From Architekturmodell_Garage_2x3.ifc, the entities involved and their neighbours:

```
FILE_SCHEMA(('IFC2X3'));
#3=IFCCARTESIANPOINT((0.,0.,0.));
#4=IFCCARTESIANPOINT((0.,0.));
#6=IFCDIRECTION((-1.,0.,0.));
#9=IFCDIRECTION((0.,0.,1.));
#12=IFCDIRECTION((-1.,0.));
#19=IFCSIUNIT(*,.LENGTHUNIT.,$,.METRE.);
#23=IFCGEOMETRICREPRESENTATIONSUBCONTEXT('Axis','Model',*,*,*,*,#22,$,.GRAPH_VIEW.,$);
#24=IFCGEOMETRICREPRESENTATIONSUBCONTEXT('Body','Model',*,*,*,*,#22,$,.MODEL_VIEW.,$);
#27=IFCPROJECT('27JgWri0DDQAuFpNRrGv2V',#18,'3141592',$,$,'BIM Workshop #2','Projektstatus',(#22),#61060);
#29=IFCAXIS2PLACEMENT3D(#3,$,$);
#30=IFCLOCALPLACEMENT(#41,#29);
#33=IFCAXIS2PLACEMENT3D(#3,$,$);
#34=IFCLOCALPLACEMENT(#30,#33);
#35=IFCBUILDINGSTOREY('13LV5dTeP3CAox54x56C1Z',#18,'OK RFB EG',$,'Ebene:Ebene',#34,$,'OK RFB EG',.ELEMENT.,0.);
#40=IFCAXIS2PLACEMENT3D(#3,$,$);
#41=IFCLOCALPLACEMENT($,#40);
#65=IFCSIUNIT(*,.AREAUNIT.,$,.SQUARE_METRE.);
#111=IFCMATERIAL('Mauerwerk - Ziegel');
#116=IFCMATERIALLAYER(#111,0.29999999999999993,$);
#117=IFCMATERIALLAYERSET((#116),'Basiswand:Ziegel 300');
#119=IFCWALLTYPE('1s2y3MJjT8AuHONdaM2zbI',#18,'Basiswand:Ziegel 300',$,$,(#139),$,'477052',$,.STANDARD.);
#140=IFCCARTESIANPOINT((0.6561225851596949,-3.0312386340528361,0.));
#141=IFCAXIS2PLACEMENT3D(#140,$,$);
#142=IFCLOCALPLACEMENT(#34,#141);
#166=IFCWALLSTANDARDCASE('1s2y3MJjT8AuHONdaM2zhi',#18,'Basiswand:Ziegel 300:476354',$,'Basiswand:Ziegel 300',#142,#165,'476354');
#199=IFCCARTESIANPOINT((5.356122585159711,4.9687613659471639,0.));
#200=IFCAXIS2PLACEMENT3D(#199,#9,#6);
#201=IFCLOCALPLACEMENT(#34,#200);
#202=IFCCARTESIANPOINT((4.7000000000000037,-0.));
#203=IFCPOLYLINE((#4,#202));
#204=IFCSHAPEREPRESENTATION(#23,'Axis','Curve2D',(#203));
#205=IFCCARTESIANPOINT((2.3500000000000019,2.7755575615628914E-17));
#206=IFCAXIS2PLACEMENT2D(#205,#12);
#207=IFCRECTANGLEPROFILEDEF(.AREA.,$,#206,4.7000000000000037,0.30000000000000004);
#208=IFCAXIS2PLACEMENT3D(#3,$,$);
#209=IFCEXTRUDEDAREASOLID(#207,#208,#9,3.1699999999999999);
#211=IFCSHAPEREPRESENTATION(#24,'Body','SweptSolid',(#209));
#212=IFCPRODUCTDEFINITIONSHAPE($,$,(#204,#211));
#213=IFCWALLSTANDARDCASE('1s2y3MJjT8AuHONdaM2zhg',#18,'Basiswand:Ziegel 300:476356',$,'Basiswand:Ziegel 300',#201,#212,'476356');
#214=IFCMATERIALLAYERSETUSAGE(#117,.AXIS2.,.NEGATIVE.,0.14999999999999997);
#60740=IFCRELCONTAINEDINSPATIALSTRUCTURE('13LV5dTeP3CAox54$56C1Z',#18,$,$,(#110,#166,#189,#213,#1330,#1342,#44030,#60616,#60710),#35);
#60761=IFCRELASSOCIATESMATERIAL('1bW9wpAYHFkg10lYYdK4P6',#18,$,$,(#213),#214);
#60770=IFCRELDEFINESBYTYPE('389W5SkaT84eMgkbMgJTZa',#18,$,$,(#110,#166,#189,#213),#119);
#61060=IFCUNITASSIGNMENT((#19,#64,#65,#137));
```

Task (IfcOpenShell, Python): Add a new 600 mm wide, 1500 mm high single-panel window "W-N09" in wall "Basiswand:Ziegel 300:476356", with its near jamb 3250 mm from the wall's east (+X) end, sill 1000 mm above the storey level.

```python
import numpy as np
import ifcopenshell
import ifcopenshell.api.feature
import ifcopenshell.api.geometry
import ifcopenshell.api.root
import ifcopenshell.api.spatial
import ifcopenshell.api.type
import ifcopenshell.geom
import ifcopenshell.util.element
import ifcopenshell.util.placement
import ifcopenshell.util.representation
import ifcopenshell.util.shape
import ifcopenshell.util.unit

model = ifcopenshell.open("Architekturmodell_Garage_2x3.ifc")
unit_scale = ifcopenshell.util.unit.calculate_unit_scale(model)
settings = ifcopenshell.geom.settings()


def volume(element):
    """Net volume in cubic metres, openings subtracted."""
    shape = ifcopenshell.geom.create_shape(settings, element)
    return ifcopenshell.util.shape.get_volume(shape.geometry)


wall = model.by_guid("1s2y3MJjT8AuHONdaM2zhg")
storey = ifcopenshell.util.element.get_container(wall, ifc_class="IfcBuildingStorey")
context = ifcopenshell.util.representation.get_context(model, "Model", "Body", "MODEL_VIEW")
before = volume(wall)

width, height, from_end, sill = 0.6, 1.5, 3.25, 1  # metres

# The wall runs along its own X axis, and the end named is its -X end.
wall_shape = ifcopenshell.geom.create_shape(settings, wall)
x, y, z = ifcopenshell.util.shape.get_vertices(wall_shape.geometry).T
start = x.min() + from_end
face, thickness = float(y.min()), float(y.max() - y.min())
wall_matrix = ifcopenshell.util.placement.get_local_placement(wall.ObjectPlacement)
level = ifcopenshell.util.placement.get_local_placement(storey.ObjectPlacement)[2, 3]


def in_wall(x, y):
    """Placement at x, y metres in the wall's axes, at sill height."""
    matrix = wall_matrix.copy()
    matrix[:, 3] = wall_matrix @ np.array([x / unit_scale, y / unit_scale, 0.0, 1.0])
    matrix[2, 3] = level + sill / unit_scale
    return matrix


# Opening: a box that overshoots both wall faces by 50 mm.
opening = ifcopenshell.api.root.create_entity(model, ifc_class="IfcOpeningElement")
box = ifcopenshell.api.geometry.add_wall_representation(
    model, context=context, length=width, height=height, thickness=thickness + 0.1
)
ifcopenshell.api.geometry.assign_representation(model, product=opening, representation=box)
ifcopenshell.api.geometry.edit_object_placement(model, product=opening, matrix=in_wall(start, face - 0.05), is_si=False)
ifcopenshell.api.feature.add_feature(model, feature=opening, element=wall)

window = ifcopenshell.api.root.create_entity(model, ifc_class="IfcWindow", name="W-N09")
window.OverallWidth, window.OverallHeight = width / unit_scale, height / unit_scale
body = ifcopenshell.api.geometry.add_window_representation(
    model,
    context=context,
    overall_width=window.OverallWidth,
    overall_height=window.OverallHeight,
    partition_type="SINGLE_PANEL",
)
ifcopenshell.api.geometry.assign_representation(model, product=window, representation=body)
ifcopenshell.api.spatial.assign_container(model, products=[window], relating_structure=storey)
fills = ifcopenshell.api.feature.add_filling(model, opening=opening, element=window)
fills.OwnerHistory = window.OwnerHistory  # required in IFC2X3

# IFC2X3 keeps the operation on the window style.
style = ifcopenshell.api.root.create_entity(model, ifc_class="IfcWindowStyle", name="W-N09")
style.OperationType, style.ConstructionType = "SINGLE_PANEL", "NOTDEFINED"
style.ParameterTakesPrecedence = style.Sizeable = False
ifcopenshell.api.type.assign_type(model, related_objects=[window], relating_type=style)

# Centre the window in the wall's thickness.
ifcopenshell.api.geometry.edit_object_placement(model, product=window, matrix=in_wall(start, face), is_si=False)
window_shape = ifcopenshell.geom.create_shape(settings, window)
depth = ifcopenshell.util.shape.get_vertices(window_shape.geometry)[:, 1]
offset = face + thickness / 2 - (depth.min() + depth.max()) / 2
ifcopenshell.api.geometry.edit_object_placement(model, product=window, matrix=in_wall(start, offset), is_si=False)

after = volume(wall)

print(f"wall volume {before:.3f} -> {after:.3f} m3")

model.write("Architekturmodell_Garage_2x3_rev.ifc")
```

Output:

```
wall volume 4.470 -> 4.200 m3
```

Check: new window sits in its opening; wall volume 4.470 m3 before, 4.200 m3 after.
